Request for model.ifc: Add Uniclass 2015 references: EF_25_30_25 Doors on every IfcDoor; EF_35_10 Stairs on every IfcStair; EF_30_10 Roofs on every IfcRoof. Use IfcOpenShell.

First a look at what the model holds.

```python
import ifcopenshell

model = ifcopenshell.open("model.ifc")
print(model.schema)
print("classifications:", [c.Name for c in model.by_type("IfcClassification")])
for ifc_class in ("IfcDoor", "IfcRoof", "IfcStair", "IfcWall", "IfcWindow"):
    print(ifc_class, len(model.by_type(ifc_class)))
```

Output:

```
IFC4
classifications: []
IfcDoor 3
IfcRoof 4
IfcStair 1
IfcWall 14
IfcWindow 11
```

```python
import ifcopenshell
import ifcopenshell.api.classification

model = ifcopenshell.open("model.ifc")

system = ifcopenshell.api.classification.add_classification(model, classification="Uniclass 2015")

codes = {
    "IfcDoor": ("EF_25_30_25", "Doors"),
    "IfcStair": ("EF_35_10", "Stairs"),
    "IfcRoof": ("EF_30_10", "Roofs"),
}
for ifc_class, (code, name) in codes.items():
    products = model.by_type(ifc_class)
    ifcopenshell.api.classification.add_reference(
        model, products=products, classification=system, identification=code, name=name
    )
    print(code, len(products))

model.write("model_v2.ifc")
```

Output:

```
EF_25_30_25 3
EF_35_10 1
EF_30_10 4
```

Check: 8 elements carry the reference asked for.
